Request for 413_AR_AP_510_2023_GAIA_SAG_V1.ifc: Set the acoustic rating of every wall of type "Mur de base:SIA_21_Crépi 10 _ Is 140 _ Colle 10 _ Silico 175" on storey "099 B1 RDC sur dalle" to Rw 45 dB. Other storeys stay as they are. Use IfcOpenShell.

First a look at what the model holds.

```python
import ifcopenshell
import ifcopenshell.util.element

model = ifcopenshell.open("413_AR_AP_510_2023_GAIA_SAG_V1.ifc")
print(model.schema)
storey = next(s for s in model.by_type("IfcBuildingStorey") if s.Name == "099 B1 RDC sur dalle")
walls = [e for e in ifcopenshell.util.element.get_decomposition(storey) if e.is_a("IfcWall")]
seen = {}
for e in walls:
    element_type = ifcopenshell.util.element.get_type(e)
    key = (element_type.Name if element_type != e and element_type else None, ifcopenshell.util.element.get_pset(e, "Pset_WallCommon", "AcousticRating"))
    seen[key] = seen.get(key, 0) + 1
for (name, value), count in sorted(seen.items(), key=str):
    print(count, "x", name, "|", value)
```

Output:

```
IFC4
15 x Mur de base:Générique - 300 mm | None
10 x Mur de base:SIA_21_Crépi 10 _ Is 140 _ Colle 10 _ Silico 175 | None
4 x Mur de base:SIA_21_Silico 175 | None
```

```python
import ifcopenshell
import ifcopenshell.api.pset
import ifcopenshell.util.element

model = ifcopenshell.open("413_AR_AP_510_2023_GAIA_SAG_V1.ifc")

storey = next(s for s in model.by_type("IfcBuildingStorey") if s.Name == "099 B1 RDC sur dalle")
walls = [e for e in ifcopenshell.util.element.get_decomposition(storey) if e.is_a("IfcWall")]

count = 0
for e in walls:
    element_type = ifcopenshell.util.element.get_type(e)
    if element_type in (None, e) or element_type.Name != "Mur de base:SIA_21_Crépi 10 _ Is 140 _ Colle 10 _ Silico 175":
        continue
    # add_pset returns the element's existing set when there is one.
    pset = ifcopenshell.api.pset.add_pset(model, product=e, name="Pset_WallCommon")
    ifcopenshell.api.pset.edit_pset(model, pset=pset, properties={"AcousticRating": "Rw 45 dB"})
    count += 1

print(count, "walls updated")

model.write("413_AR_AP_510_2023_GAIA_SAG_V1_edited.ifc")
```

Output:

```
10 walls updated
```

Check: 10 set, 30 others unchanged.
